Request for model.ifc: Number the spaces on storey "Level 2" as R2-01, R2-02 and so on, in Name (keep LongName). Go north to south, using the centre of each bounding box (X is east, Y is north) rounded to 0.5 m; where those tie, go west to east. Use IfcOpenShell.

First a look at what the model holds.

```python
import ifcopenshell
import ifcopenshell.util.element
import ifcopenshell.util.placement

model = ifcopenshell.open("model.ifc")
print(model.schema)
storey = next(s for s in model.by_type("IfcBuildingStorey") if s.Name == "Level 2")
spaces = [e for e in ifcopenshell.util.element.get_decomposition(storey) if e.is_a("IfcSpace")]
for e in sorted(spaces, key=lambda e: e.id()):
    origin = ifcopenshell.util.placement.get_local_placement(e.ObjectPlacement)[:3, 3]
    print(e.id(), e.Name, e.LongName, origin.round(2) + 0.0, sep=" | ")
```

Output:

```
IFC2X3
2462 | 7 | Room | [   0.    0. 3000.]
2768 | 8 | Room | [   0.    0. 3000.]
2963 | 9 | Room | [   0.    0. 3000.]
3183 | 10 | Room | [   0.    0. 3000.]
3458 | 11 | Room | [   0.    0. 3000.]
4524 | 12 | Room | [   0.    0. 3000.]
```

```python
import ifcopenshell
import ifcopenshell.geom
import ifcopenshell.util.element
import ifcopenshell.util.shape

model = ifcopenshell.open("model.ifc")
settings = ifcopenshell.geom.settings()
settings.set("use-world-coords", True)


def centre(element):
    shape = ifcopenshell.geom.create_shape(settings, element)
    return ifcopenshell.util.shape.get_bbox_centroid(shape.geometry)


storey = next(s for s in model.by_type("IfcBuildingStorey") if s.Name == "Level 2")
spaces = [e for e in ifcopenshell.util.element.get_decomposition(storey) if e.is_a("IfcSpace")]

# Insertion points can sit at a corner or the storey origin, so sort by the geometry (in metres).
centres = {e: centre(e) for e in spaces}
spaces.sort(key=lambda e: (-round(centres[e][1] / 0.5), centres[e][0]))

for i, e in enumerate(spaces, start=1):
    number = f"R2-{i:02d}"
    e.Name = number
    print(e.id(), number)

model.write("model_edited.ifc")
```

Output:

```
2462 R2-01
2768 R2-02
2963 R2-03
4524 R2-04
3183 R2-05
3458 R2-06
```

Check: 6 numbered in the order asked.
